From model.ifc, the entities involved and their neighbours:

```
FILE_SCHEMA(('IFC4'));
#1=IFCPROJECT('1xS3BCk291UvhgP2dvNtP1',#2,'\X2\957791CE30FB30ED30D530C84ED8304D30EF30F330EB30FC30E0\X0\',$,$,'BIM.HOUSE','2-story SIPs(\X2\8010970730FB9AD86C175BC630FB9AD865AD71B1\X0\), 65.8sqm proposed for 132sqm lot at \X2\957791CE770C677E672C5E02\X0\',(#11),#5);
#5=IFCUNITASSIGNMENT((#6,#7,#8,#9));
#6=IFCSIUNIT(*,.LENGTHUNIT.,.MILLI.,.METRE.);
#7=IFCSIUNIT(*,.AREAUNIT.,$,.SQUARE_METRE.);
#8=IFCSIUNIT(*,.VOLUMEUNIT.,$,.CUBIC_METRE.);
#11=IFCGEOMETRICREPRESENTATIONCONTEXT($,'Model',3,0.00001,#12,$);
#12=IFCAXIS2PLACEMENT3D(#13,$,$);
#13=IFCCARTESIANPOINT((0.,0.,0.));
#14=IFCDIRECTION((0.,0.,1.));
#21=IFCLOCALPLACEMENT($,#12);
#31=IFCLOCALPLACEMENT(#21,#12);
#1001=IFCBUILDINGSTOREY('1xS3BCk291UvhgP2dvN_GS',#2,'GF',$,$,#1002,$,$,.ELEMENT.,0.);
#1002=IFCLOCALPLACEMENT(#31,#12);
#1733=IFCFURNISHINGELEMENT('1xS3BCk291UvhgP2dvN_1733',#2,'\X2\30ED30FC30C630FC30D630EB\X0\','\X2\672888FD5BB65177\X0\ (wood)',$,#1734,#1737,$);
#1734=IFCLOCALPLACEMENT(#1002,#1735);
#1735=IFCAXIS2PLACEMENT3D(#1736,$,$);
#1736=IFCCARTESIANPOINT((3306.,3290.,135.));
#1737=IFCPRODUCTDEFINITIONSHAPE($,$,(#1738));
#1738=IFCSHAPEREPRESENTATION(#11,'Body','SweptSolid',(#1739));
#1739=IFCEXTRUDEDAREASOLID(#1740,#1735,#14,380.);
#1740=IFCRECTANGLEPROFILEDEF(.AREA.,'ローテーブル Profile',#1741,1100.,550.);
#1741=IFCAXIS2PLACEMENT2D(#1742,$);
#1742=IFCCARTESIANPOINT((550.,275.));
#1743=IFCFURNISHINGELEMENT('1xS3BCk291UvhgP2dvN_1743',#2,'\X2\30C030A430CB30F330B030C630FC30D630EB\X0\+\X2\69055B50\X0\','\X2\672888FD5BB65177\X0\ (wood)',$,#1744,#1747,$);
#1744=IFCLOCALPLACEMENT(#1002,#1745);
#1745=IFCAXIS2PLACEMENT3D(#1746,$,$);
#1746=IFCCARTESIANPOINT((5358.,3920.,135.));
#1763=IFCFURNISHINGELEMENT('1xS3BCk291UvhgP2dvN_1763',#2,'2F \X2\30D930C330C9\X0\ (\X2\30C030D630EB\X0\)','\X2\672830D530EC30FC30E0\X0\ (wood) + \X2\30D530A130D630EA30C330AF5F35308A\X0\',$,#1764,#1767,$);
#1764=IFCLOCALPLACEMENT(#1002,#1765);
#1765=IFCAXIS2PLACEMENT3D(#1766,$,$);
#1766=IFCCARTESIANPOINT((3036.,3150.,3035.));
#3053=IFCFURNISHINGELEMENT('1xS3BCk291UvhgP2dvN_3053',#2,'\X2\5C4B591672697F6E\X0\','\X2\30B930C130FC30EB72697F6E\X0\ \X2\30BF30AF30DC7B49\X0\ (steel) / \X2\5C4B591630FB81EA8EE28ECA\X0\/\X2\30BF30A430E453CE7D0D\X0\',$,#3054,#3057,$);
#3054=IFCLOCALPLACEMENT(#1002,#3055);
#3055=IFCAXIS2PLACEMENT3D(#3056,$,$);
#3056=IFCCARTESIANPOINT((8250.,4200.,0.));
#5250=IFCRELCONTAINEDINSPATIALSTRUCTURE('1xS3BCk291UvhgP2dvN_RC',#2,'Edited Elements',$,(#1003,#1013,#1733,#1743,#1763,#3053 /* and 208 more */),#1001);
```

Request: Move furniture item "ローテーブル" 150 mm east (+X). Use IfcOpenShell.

```python
import ifcopenshell
import ifcopenshell.api.geometry
import ifcopenshell.util.placement
import ifcopenshell.util.unit

model = ifcopenshell.open("model.ifc")
unit_scale = ifcopenshell.util.unit.calculate_unit_scale(model)

item = model.by_id(1733)
matrix = ifcopenshell.util.placement.get_local_placement(item.ObjectPlacement)
matrix[0, 3] += 0.15 / unit_scale
ifcopenshell.api.geometry.edit_object_placement(model, product=item, matrix=matrix, is_si=False)

print(ifcopenshell.util.placement.get_local_placement(item.ObjectPlacement).round(3) + 0.0)

model.write("model_edited.ifc")
```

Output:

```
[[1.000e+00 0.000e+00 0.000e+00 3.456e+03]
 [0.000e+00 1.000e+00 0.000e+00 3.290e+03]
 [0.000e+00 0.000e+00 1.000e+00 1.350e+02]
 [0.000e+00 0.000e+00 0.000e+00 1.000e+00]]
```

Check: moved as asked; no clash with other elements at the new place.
